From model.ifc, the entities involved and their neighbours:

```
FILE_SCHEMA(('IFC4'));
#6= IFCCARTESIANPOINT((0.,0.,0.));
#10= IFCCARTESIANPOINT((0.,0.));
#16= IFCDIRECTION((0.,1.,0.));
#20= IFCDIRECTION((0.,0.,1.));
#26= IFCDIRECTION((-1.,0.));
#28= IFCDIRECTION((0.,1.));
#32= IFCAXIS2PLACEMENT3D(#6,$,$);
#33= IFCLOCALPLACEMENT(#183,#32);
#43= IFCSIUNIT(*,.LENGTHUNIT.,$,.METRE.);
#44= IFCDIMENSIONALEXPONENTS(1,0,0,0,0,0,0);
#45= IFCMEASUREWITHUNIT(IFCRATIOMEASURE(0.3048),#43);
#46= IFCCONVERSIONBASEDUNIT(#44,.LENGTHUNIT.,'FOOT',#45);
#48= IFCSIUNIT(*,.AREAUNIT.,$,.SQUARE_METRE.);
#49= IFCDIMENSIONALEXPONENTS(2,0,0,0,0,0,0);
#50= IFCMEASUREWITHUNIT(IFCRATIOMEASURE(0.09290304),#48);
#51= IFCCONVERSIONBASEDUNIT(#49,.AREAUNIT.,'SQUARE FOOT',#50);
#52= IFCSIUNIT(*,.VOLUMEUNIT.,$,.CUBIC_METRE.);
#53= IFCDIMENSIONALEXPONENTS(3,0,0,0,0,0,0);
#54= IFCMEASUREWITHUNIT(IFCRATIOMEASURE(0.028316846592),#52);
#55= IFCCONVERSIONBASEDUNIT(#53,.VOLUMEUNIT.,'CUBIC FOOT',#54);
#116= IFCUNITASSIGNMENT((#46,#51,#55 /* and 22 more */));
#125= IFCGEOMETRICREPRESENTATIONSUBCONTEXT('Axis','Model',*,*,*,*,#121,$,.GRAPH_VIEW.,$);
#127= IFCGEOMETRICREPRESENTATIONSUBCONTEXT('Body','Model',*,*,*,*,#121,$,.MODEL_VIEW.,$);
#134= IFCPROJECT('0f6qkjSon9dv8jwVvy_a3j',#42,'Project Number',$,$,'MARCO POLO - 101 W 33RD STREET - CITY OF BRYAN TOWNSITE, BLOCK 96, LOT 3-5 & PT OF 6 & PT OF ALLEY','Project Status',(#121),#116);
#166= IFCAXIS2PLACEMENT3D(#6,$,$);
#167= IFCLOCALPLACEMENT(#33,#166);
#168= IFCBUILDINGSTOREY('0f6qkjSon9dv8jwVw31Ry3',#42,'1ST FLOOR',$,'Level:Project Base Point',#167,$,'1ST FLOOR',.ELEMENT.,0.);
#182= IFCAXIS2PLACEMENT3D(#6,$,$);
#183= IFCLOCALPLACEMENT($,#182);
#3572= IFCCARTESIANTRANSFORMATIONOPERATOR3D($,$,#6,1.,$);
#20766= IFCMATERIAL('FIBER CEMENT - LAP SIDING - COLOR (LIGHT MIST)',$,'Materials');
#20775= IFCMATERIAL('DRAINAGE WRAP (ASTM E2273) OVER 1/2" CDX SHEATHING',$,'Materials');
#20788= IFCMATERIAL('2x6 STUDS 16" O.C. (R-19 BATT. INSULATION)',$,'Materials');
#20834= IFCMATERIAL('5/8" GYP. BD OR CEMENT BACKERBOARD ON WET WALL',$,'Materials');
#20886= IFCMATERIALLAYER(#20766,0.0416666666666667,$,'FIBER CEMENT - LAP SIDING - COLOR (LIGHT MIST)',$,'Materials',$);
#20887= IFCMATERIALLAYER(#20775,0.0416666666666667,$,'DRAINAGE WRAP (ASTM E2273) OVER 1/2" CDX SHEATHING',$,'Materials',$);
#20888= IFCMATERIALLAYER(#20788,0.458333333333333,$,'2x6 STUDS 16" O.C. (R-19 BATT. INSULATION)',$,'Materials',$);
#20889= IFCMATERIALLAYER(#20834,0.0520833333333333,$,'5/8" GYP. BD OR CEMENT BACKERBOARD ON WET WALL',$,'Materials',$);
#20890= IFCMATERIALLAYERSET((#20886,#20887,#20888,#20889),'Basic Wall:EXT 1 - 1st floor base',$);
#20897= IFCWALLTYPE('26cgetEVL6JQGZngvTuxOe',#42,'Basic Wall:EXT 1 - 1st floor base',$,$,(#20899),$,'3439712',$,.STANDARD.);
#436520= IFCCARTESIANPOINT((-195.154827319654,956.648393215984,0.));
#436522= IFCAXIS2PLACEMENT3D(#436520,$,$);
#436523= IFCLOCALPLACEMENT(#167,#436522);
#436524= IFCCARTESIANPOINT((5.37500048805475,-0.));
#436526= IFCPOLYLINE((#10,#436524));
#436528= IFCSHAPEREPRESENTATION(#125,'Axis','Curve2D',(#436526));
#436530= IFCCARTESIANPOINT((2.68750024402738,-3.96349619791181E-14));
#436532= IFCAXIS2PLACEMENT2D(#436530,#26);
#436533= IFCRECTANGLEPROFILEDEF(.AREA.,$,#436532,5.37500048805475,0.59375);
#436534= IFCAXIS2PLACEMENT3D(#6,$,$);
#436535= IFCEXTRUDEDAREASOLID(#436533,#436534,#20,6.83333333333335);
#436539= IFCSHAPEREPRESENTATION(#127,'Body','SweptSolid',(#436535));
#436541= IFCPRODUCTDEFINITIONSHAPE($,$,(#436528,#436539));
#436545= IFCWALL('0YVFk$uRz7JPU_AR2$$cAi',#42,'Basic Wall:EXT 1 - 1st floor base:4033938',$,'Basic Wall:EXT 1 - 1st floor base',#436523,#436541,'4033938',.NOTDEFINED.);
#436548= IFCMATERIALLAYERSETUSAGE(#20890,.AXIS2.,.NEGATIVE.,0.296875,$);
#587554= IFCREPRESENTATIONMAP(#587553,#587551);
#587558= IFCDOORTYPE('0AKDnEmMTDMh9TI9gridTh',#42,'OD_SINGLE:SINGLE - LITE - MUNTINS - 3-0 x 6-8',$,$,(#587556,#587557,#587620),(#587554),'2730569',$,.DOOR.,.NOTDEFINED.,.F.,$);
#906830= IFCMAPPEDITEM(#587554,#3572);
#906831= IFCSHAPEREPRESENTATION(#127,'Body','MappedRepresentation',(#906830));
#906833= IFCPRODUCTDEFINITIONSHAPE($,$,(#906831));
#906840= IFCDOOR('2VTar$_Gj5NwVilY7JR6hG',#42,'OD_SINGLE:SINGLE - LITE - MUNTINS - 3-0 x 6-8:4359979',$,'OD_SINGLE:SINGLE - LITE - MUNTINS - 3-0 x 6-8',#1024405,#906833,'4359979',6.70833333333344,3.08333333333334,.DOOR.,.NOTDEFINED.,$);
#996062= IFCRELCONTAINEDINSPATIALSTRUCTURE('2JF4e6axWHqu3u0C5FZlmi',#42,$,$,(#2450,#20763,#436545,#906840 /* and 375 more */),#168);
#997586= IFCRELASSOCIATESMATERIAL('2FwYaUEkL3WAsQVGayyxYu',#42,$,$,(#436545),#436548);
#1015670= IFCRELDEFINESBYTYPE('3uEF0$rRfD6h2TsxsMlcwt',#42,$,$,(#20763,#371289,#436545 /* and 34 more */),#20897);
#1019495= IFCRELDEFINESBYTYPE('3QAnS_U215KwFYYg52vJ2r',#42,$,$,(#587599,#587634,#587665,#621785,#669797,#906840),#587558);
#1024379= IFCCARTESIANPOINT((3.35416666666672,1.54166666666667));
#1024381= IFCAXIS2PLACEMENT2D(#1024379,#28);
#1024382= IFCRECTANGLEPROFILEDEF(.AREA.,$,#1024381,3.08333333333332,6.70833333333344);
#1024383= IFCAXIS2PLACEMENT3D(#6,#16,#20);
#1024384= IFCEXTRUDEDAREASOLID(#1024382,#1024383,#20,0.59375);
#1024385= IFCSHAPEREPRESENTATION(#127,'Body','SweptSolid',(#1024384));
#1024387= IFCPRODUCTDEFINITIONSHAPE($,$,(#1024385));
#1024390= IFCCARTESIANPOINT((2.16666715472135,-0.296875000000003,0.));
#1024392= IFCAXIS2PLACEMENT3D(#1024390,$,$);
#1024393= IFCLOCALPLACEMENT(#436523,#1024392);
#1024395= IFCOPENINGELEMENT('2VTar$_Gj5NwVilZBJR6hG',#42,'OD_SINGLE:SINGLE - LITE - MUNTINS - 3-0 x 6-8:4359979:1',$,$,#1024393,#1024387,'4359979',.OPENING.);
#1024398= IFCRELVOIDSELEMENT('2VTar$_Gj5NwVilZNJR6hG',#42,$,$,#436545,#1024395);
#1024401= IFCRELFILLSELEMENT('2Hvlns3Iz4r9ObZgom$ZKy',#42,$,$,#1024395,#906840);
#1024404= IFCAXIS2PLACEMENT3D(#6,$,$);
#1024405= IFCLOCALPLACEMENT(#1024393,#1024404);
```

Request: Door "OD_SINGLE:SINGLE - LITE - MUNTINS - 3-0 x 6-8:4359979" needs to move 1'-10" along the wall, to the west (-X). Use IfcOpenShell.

```python
import ifcopenshell
import ifcopenshell.api.geometry
import ifcopenshell.util.placement
import ifcopenshell.util.unit

model = ifcopenshell.open("model.ifc")
unit_scale = ifcopenshell.util.unit.calculate_unit_scale(model)

door = model.by_guid("2VTar$_Gj5NwVilY7JR6hG")
opening = door.FillsVoids[0].RelatingOpeningElement
wall = opening.VoidsElements[0].RelatingBuildingElement

wall_matrix = ifcopenshell.util.placement.get_local_placement(wall.ObjectPlacement)
shift = wall_matrix[:3, 0] * -22 * 0.0254 / unit_scale
before = ifcopenshell.util.placement.get_local_placement(door.ObjectPlacement)[:3, 3].copy()

# The door is placed relative to its opening, so it follows when the opening moves.
matrix = ifcopenshell.util.placement.get_local_placement(opening.ObjectPlacement)
matrix[:3, 3] += shift
ifcopenshell.api.geometry.edit_object_placement(
    model, product=opening, matrix=matrix, is_si=False, should_transform_children=True
)

after = ifcopenshell.util.placement.get_local_placement(door.ObjectPlacement)[:3, 3]
print("door moved by", (after - before).round(3) + 0.0)

model.write("model_edited.ifc")
```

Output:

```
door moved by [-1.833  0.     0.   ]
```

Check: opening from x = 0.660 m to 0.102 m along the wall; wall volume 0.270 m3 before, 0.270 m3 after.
